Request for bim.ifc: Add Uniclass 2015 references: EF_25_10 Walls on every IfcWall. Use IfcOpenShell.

First a look at what the model holds.

```python
import ifcopenshell

model = ifcopenshell.open("bim.ifc")
print(model.schema)
print("classifications:", [c.Name for c in model.by_type("IfcClassification")])
for ifc_class in ("IfcDoor", "IfcRoof", "IfcStair", "IfcWall", "IfcWindow"):
    print(ifc_class, len(model.by_type(ifc_class)))
```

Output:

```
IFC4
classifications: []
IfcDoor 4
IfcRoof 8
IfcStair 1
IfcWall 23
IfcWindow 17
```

```python
import ifcopenshell
import ifcopenshell.api.classification

model = ifcopenshell.open("bim.ifc")

system = ifcopenshell.api.classification.add_classification(model, classification="Uniclass 2015")

codes = {
    "IfcWall": ("EF_25_10", "Walls"),
}
for ifc_class, (code, name) in codes.items():
    products = model.by_type(ifc_class)
    ifcopenshell.api.classification.add_reference(
        model, products=products, classification=system, identification=code, name=name
    )
    print(code, len(products))

model.write("bim_edited.ifc")
```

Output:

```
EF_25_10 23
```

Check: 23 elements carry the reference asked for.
